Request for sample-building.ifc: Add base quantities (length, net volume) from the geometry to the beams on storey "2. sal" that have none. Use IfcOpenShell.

First a look at what the model holds.

```python
import ifcopenshell
import ifcopenshell.util.element
import ifcopenshell.util.unit

model = ifcopenshell.open("sample-building.ifc")
print(model.schema)
for unit_type in ("LENGTHUNIT", "AREAUNIT", "VOLUMEUNIT"):
    print(unit_type, ifcopenshell.util.unit.calculate_unit_scale(model, unit_type))
storey = next(s for s in model.by_type("IfcBuildingStorey") if s.Name == "2. sal")
beams = [e for e in ifcopenshell.util.element.get_decomposition(storey) if e.is_a("IfcBeam")]
for e in sorted(beams, key=lambda e: e.id()):
    print(e.id(), e.is_a(), e.Name, list(ifcopenshell.util.element.get_psets(e, qtos_only=True)), sep=" | ")
```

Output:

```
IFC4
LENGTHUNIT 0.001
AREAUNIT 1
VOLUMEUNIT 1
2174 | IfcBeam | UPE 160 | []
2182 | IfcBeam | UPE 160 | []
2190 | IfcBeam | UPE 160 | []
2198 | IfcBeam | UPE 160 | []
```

```python
import ifcopenshell
import ifcopenshell.api.pset
import ifcopenshell.geom
import ifcopenshell.util.element
import ifcopenshell.util.shape
import ifcopenshell.util.unit

model = ifcopenshell.open("sample-building.ifc")
unit_scale = ifcopenshell.util.unit.calculate_unit_scale(model)
volume_scale = ifcopenshell.util.unit.calculate_unit_scale(model, "VOLUMEUNIT")
settings = ifcopenshell.geom.settings()

storey = next(s for s in model.by_type("IfcBuildingStorey") if s.Name == "2. sal")
beams = [e for e in ifcopenshell.util.element.get_decomposition(storey) if e.is_a("IfcBeam")]

for e in sorted(beams, key=lambda e: e.id()):
    if ifcopenshell.util.element.get_psets(e, qtos_only=True, should_inherit=False):
        continue
    # Geometry comes back in metres, in the element's own axes.
    shape = ifcopenshell.geom.create_shape(settings, e)
    values = {
        "Length": ifcopenshell.util.shape.get_max_xyz(shape.geometry) / unit_scale,
        "NetVolume": ifcopenshell.util.shape.get_volume(shape.geometry) / volume_scale,
    }
    qto = ifcopenshell.api.pset.add_qto(model, product=e, name="Qto_BeamBaseQuantities")
    ifcopenshell.api.pset.edit_qto(model, qto=qto, properties=values)
    print(e.id(), {k: round(v, 3) for k, v in values.items()})

model.write("sample-building-out.ifc")
```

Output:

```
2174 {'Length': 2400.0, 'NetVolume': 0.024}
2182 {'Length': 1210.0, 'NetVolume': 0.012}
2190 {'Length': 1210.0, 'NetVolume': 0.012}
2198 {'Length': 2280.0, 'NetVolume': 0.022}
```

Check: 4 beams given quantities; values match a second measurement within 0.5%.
